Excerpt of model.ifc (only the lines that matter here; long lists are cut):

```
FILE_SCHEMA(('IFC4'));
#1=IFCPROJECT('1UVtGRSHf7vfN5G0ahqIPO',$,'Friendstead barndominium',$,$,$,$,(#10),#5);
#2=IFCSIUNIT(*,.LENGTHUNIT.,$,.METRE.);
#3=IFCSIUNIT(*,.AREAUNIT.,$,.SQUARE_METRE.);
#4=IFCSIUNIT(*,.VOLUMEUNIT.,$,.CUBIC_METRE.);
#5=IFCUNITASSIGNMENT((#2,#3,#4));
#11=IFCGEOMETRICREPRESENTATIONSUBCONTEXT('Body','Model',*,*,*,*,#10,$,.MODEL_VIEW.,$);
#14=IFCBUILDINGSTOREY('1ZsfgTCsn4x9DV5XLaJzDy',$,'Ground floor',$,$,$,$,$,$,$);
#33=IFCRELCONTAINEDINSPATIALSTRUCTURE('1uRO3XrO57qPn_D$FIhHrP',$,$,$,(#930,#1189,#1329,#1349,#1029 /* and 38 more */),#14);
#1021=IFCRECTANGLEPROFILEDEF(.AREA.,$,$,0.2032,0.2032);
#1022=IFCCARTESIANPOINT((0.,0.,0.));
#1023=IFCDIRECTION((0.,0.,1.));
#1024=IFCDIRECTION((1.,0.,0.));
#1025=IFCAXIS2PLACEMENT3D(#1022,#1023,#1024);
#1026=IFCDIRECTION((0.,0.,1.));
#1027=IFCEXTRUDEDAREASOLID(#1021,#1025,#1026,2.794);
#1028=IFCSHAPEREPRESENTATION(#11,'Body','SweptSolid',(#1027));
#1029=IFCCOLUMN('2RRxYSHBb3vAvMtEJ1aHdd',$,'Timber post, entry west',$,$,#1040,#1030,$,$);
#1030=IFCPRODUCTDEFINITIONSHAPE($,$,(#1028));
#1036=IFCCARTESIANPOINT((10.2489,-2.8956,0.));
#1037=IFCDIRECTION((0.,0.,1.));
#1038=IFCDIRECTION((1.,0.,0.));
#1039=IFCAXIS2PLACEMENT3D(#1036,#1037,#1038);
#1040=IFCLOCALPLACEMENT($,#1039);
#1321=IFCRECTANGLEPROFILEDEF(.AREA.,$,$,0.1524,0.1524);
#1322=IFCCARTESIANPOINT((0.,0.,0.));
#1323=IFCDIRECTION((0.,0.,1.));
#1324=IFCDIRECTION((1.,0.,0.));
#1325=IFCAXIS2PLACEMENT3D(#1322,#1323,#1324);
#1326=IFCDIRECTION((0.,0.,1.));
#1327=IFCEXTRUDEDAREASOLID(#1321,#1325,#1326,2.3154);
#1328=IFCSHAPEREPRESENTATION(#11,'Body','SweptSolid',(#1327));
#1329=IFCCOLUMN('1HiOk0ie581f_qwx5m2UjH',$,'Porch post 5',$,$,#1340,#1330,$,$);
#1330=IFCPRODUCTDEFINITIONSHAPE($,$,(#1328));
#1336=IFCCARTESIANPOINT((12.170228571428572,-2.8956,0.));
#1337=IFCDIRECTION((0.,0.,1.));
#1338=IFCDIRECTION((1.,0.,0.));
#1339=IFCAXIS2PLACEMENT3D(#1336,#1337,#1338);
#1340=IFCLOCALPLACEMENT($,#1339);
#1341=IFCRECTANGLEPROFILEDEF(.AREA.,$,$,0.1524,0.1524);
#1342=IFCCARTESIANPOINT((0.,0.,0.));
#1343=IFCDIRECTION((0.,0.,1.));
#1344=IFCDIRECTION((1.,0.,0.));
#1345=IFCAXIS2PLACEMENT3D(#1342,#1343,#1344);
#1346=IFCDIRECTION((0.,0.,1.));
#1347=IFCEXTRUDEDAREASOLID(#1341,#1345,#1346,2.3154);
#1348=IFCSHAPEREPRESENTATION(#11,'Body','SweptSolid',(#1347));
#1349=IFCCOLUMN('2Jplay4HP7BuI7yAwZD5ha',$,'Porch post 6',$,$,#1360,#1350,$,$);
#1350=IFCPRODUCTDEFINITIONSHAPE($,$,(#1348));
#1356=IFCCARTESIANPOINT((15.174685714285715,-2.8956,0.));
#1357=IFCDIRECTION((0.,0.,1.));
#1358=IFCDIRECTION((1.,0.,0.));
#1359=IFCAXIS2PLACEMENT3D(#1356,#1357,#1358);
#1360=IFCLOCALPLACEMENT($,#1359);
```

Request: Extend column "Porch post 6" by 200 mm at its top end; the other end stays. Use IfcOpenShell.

```python
import ifcopenshell
import ifcopenshell.util.representation

model = ifcopenshell.open("model.ifc")

member = model.by_guid("2Jplay4HP7BuI7yAwZD5ha")
change = 0.2

# The extrusion runs towards the end named, so only its depth changes.
body = ifcopenshell.util.representation.get_representation(member, "Model", "Body")
solid = body.Items[0]
old_length = solid.Depth
solid.Depth += change

print(f"length {old_length:g} -> {solid.Depth:g}")

model.write("model_v2.ifc")
```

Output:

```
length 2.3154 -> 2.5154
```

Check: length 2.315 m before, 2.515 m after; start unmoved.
